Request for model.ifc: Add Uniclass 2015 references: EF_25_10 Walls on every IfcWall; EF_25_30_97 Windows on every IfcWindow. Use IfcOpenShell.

First a look at what the model holds.

```python
import ifcopenshell

model = ifcopenshell.open("model.ifc")
print(model.schema)
print("classifications:", [c.Name for c in model.by_type("IfcClassification")])
for ifc_class in ("IfcDoor", "IfcRoof", "IfcStair", "IfcWall", "IfcWindow"):
    print(ifc_class, len(model.by_type(ifc_class)))
```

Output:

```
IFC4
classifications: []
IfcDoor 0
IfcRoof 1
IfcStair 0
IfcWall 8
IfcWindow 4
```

```python
import ifcopenshell
import ifcopenshell.api.classification

model = ifcopenshell.open("model.ifc")

system = ifcopenshell.api.classification.add_classification(model, classification="Uniclass 2015")

codes = {
    "IfcWall": ("EF_25_10", "Walls"),
    "IfcWindow": ("EF_25_30_97", "Windows"),
}
for ifc_class, (code, name) in codes.items():
    products = model.by_type(ifc_class)
    ifcopenshell.api.classification.add_reference(
        model, products=products, classification=system, identification=code, name=name
    )
    print(code, len(products))

model.write("model_rev.ifc")
```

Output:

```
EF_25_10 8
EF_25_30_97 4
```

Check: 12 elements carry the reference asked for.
